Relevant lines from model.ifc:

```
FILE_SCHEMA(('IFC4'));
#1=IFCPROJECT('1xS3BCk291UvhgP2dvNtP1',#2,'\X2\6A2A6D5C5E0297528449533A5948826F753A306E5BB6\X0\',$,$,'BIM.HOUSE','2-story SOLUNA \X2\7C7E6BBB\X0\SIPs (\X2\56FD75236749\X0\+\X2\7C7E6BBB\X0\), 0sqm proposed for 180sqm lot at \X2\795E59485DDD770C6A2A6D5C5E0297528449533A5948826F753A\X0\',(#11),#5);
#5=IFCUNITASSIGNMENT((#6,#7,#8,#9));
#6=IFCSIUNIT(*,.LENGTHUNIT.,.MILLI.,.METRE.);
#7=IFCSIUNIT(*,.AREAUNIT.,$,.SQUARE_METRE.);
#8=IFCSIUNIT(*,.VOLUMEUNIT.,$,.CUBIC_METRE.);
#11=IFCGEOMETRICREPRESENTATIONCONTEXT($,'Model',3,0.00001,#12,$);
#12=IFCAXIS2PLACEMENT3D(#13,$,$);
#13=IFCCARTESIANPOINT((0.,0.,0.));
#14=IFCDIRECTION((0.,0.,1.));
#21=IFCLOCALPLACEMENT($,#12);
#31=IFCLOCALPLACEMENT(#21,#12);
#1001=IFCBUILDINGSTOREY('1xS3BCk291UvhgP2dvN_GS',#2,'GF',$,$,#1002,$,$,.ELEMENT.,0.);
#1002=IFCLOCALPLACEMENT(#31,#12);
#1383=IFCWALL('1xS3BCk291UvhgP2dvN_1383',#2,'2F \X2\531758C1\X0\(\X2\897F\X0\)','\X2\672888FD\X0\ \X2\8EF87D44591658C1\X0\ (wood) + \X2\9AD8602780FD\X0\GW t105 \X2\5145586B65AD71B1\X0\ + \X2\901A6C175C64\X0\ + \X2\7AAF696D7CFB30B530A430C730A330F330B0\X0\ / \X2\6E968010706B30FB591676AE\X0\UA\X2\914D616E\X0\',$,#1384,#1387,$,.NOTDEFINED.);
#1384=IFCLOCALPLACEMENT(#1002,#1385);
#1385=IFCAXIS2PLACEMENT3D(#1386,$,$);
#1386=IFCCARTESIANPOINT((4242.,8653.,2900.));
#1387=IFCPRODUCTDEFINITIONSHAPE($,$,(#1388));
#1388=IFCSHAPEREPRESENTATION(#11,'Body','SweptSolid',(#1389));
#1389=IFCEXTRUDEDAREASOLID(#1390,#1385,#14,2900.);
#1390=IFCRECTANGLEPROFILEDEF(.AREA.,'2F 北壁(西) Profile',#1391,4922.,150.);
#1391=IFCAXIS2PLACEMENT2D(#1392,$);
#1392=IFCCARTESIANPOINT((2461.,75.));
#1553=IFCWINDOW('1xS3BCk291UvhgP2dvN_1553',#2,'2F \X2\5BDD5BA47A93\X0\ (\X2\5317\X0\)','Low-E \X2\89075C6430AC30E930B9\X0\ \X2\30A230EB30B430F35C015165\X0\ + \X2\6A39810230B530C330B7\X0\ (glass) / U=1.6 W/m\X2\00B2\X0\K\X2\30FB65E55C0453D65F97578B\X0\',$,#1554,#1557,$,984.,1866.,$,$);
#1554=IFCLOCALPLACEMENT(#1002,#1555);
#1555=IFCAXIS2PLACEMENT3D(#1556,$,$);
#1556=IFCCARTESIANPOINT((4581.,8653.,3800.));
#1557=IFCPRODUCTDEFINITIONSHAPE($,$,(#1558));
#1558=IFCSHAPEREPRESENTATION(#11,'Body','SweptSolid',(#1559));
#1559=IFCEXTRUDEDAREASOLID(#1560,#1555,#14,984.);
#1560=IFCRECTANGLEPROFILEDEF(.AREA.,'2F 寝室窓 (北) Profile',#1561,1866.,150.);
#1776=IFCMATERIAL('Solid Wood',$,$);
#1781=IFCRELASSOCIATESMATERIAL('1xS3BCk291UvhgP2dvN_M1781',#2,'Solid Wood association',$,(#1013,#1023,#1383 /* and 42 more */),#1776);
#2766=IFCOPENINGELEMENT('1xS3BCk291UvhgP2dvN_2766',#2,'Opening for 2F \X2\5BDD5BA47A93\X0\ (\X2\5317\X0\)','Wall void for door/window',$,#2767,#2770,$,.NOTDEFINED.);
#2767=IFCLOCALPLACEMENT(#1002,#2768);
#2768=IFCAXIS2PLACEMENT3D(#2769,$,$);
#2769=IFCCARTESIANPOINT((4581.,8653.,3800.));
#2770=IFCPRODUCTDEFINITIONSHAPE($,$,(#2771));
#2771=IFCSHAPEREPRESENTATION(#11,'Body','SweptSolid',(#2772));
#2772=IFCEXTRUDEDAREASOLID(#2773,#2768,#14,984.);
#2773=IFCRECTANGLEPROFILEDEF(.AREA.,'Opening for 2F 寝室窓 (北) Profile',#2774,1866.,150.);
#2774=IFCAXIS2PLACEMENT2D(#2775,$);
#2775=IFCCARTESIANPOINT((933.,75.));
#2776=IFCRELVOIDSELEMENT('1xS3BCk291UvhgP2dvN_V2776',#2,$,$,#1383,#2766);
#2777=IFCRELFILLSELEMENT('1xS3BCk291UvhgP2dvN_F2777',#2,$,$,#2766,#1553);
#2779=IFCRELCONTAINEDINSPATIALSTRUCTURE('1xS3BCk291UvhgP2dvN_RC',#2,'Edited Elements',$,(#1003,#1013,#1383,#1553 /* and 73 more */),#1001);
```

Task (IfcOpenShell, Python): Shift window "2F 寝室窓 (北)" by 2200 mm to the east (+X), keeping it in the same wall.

```python
import ifcopenshell
import ifcopenshell.api.geometry
import ifcopenshell.util.placement
import ifcopenshell.util.unit

model = ifcopenshell.open("model.ifc")
unit_scale = ifcopenshell.util.unit.calculate_unit_scale(model)

window = model.by_guid("1xS3BCk291UvhgP2dvN_1553")
opening = window.FillsVoids[0].RelatingOpeningElement
wall = opening.VoidsElements[0].RelatingBuildingElement

wall_matrix = ifcopenshell.util.placement.get_local_placement(wall.ObjectPlacement)
shift = wall_matrix[:3, 0] * 2.2 / unit_scale
before = ifcopenshell.util.placement.get_local_placement(window.ObjectPlacement)[:3, 3].copy()

# The window is not placed relative to its opening, so move both.
for product in (opening, window):
    matrix = ifcopenshell.util.placement.get_local_placement(product.ObjectPlacement)
    matrix[:3, 3] += shift
    ifcopenshell.api.geometry.edit_object_placement(model, product=product, matrix=matrix, is_si=False)

after = ifcopenshell.util.placement.get_local_placement(window.ObjectPlacement)[:3, 3]
print("window moved by", (after - before).round(3) + 0.0)

model.write("model-out.ifc")
```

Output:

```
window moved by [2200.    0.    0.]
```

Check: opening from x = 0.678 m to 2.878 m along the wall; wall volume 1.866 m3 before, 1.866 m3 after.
